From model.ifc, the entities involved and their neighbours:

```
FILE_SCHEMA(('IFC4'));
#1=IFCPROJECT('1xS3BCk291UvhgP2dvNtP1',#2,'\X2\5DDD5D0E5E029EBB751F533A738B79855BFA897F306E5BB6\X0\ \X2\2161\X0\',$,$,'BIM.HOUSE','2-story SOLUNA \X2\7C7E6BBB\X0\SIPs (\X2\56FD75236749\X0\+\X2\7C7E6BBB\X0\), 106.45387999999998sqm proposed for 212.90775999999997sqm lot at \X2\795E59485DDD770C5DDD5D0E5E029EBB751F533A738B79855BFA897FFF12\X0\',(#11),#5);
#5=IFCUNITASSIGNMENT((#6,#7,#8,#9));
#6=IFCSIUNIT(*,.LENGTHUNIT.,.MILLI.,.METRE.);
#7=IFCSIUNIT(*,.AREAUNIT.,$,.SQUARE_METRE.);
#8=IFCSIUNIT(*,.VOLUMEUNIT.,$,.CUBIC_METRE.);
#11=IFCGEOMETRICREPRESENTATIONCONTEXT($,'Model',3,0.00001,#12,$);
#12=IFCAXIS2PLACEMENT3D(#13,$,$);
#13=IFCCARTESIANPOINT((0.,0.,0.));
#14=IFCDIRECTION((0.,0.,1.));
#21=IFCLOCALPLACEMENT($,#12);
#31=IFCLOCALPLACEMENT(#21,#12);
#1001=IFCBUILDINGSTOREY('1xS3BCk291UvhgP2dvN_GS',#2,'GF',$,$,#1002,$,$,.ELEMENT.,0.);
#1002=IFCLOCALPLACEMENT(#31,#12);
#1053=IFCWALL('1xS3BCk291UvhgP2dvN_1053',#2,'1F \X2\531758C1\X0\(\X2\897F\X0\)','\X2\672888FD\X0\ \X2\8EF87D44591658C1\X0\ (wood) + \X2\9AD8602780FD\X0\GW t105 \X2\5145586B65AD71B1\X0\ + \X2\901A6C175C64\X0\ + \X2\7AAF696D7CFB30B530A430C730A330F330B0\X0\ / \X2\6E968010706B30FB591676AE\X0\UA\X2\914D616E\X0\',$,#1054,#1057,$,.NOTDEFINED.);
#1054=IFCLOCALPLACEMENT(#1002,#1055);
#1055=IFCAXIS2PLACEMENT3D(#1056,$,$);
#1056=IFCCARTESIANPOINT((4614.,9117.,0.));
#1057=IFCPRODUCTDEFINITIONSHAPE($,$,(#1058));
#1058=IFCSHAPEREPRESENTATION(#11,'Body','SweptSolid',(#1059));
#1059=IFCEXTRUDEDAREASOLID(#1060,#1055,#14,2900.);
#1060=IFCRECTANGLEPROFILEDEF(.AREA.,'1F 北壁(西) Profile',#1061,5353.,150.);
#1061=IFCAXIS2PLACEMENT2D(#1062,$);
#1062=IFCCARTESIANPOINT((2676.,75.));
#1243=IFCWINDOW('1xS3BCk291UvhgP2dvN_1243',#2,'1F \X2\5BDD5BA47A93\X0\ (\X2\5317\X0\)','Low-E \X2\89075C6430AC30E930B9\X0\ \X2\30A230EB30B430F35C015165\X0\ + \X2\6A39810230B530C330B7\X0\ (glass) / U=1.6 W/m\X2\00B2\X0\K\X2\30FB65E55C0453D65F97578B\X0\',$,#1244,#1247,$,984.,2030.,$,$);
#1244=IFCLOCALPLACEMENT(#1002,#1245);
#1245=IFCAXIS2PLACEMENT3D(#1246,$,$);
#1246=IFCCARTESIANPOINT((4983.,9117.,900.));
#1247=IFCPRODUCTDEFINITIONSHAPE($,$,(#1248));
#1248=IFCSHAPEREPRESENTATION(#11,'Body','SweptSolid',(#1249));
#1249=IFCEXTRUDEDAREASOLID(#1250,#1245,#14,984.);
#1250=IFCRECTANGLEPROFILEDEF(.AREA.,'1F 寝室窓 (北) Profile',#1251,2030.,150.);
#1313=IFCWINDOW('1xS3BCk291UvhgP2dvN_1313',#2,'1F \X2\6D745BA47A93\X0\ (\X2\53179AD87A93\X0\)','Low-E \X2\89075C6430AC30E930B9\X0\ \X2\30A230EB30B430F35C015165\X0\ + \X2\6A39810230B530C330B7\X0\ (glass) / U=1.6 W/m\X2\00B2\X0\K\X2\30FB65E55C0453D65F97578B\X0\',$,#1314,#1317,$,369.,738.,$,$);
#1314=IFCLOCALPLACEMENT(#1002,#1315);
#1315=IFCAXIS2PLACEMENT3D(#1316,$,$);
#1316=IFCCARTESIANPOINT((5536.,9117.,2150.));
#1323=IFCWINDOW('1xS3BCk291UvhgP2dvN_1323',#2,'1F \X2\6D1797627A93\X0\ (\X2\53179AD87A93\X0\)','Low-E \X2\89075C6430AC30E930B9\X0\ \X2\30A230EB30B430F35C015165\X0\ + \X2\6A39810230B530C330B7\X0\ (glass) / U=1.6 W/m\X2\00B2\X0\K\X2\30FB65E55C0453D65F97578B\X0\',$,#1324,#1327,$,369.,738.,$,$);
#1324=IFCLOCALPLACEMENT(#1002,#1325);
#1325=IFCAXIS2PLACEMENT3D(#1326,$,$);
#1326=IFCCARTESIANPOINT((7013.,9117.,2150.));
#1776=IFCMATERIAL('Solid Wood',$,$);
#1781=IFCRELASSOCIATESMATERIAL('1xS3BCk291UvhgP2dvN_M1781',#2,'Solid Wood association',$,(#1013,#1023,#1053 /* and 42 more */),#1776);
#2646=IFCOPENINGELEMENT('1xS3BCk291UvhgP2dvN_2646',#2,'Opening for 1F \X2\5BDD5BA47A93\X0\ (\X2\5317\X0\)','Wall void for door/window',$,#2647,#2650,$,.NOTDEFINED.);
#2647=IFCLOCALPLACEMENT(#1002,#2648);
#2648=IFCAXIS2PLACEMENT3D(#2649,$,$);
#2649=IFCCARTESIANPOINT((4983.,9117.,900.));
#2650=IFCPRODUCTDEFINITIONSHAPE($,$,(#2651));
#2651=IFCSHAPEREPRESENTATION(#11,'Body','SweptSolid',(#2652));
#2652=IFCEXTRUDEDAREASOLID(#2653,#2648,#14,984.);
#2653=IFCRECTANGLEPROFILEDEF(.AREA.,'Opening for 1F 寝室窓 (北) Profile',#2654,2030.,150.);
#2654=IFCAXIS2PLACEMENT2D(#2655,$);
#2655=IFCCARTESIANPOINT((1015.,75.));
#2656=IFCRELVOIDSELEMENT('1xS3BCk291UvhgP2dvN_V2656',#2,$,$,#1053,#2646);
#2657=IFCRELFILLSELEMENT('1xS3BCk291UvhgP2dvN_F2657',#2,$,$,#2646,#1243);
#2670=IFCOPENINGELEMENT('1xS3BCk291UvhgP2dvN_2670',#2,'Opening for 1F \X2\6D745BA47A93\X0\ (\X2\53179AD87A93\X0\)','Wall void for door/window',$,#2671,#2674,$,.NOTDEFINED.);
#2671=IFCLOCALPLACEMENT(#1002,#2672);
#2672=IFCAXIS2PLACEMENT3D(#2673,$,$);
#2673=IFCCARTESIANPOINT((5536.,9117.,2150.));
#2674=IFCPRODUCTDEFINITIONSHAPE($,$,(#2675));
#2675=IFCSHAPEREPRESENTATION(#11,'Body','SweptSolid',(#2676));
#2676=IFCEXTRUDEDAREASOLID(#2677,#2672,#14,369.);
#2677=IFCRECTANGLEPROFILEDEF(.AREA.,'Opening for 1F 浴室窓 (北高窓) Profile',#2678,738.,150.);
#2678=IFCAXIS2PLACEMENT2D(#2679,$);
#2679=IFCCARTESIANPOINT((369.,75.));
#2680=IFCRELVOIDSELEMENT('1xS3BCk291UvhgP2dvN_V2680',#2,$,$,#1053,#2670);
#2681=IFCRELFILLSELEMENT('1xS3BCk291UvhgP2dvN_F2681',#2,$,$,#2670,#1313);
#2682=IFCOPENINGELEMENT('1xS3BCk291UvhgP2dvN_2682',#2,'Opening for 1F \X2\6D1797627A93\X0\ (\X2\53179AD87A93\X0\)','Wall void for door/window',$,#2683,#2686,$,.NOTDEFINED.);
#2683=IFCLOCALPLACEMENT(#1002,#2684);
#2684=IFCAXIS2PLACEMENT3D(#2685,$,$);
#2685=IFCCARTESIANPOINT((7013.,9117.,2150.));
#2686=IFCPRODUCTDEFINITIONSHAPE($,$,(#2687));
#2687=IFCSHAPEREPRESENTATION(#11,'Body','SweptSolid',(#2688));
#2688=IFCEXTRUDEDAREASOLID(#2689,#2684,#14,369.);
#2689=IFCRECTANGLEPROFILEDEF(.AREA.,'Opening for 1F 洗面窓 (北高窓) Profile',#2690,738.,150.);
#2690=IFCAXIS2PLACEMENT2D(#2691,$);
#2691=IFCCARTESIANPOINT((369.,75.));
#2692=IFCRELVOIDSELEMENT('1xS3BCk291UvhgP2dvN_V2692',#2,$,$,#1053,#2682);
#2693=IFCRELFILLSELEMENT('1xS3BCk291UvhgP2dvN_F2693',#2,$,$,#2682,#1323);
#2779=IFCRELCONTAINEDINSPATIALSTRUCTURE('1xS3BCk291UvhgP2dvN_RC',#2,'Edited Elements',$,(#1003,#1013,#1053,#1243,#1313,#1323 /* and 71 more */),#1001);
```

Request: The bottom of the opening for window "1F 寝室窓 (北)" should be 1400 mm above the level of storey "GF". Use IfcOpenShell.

```python
import numpy as np
import ifcopenshell
import ifcopenshell.api.geometry
import ifcopenshell.geom
import ifcopenshell.util.element
import ifcopenshell.util.placement
import ifcopenshell.util.shape
import ifcopenshell.util.unit

model = ifcopenshell.open("model.ifc")
unit_scale = ifcopenshell.util.unit.calculate_unit_scale(model)

window = model.by_id(1243)
opening = window.FillsVoids[0].RelatingOpeningElement
storey = ifcopenshell.util.element.get_container(window, ifc_class="IfcBuildingStorey")
level = ifcopenshell.util.placement.get_local_placement(storey.ObjectPlacement)[2, 3]

# The opening's origin need not be at the sill, so measure its lowest point.
shape = ifcopenshell.geom.create_shape(ifcopenshell.geom.settings(), opening)
bottom = ifcopenshell.util.shape.get_shape_bottom_elevation(shape, shape.geometry) / unit_scale
dz = level + 1.4 / unit_scale - bottom

shift = np.array([0.0, 0.0, dz])
# The window is not placed relative to its opening, so move both.
for product in (opening, window):
    matrix = ifcopenshell.util.placement.get_local_placement(product.ObjectPlacement)
    matrix[:3, 3] += shift
    ifcopenshell.api.geometry.edit_object_placement(model, product=product, matrix=matrix, is_si=False)

print(f"moved by {dz * unit_scale:+.3f} m")

model.write("model_updated.ifc")
```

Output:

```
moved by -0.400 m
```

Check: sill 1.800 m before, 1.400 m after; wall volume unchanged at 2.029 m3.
